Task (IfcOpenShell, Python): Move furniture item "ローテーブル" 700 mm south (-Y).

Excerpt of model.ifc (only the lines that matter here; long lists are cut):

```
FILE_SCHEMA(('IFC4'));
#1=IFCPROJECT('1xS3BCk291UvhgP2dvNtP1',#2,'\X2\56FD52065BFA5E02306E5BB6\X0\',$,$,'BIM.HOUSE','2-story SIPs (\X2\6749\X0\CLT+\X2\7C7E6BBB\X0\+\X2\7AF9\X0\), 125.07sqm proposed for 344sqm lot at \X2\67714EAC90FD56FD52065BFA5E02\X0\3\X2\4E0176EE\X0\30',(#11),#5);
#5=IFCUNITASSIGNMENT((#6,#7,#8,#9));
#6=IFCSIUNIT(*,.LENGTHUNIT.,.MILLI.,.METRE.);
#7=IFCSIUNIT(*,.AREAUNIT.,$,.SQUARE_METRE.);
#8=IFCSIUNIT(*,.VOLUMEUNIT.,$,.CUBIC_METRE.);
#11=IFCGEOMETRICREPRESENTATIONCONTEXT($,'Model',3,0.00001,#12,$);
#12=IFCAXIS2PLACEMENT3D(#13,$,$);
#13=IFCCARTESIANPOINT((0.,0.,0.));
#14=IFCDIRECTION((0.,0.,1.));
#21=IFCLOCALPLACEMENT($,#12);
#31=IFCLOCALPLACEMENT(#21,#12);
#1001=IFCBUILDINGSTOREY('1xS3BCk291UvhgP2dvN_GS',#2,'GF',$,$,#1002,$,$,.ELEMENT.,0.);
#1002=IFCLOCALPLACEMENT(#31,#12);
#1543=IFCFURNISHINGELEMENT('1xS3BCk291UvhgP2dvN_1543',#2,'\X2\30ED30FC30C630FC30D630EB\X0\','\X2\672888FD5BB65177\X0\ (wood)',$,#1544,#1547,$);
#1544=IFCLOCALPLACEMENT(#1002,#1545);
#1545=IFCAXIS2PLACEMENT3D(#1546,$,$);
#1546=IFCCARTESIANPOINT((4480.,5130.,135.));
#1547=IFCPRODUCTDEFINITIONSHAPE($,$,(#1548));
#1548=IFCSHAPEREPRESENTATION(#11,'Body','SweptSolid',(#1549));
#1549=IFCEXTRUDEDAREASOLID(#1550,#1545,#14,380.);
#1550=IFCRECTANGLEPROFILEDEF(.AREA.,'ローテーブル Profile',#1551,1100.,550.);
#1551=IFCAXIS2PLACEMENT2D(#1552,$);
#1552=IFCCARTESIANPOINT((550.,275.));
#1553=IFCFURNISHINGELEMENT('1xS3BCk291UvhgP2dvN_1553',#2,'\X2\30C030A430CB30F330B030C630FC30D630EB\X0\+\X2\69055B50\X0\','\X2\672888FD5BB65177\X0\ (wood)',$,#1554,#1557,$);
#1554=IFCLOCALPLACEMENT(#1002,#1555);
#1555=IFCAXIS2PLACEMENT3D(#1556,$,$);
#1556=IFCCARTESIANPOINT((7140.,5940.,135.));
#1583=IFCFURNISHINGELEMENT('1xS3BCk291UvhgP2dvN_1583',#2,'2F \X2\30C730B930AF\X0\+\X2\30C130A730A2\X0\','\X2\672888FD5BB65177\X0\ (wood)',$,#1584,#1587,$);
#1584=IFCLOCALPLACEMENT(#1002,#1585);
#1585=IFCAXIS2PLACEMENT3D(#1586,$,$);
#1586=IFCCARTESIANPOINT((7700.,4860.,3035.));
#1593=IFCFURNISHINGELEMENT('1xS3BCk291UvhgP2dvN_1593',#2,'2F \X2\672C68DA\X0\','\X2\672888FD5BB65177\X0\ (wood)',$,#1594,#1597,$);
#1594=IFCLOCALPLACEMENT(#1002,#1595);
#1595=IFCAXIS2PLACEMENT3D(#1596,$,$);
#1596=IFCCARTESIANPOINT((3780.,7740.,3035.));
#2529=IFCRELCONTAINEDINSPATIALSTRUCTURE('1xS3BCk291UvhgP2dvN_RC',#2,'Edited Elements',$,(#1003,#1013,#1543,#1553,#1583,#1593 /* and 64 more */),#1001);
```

```python
import ifcopenshell
import ifcopenshell.api.geometry
import ifcopenshell.util.placement

model = ifcopenshell.open("model.ifc")

item = model.by_guid("1xS3BCk291UvhgP2dvN_1543")
matrix = ifcopenshell.util.placement.get_local_placement(item.ObjectPlacement)
matrix[1, 3] -= 700.0
ifcopenshell.api.geometry.edit_object_placement(model, product=item, matrix=matrix, is_si=False)

print(ifcopenshell.util.placement.get_local_placement(item.ObjectPlacement).round(3) + 0.0)

model.write("model_rev.ifc")
```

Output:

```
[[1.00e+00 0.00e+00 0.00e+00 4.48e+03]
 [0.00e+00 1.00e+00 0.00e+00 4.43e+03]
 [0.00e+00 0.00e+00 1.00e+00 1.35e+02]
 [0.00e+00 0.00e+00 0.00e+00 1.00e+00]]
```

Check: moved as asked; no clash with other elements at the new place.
